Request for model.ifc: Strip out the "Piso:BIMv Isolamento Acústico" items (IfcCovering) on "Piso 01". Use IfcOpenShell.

First a look at what the model holds.

```python
import ifcopenshell
import ifcopenshell.util.element

model = ifcopenshell.open("model.ifc")
print(model.schema)
storey = next(s for s in model.by_type("IfcBuildingStorey") if s.Name == "Piso 01")
coverings = [e for e in ifcopenshell.util.element.get_decomposition(storey) if e.is_a("IfcCovering")]
seen = {}
for e in coverings:
    element_type = ifcopenshell.util.element.get_type(e)
    name = element_type.Name if element_type not in (None, e) else None
    seen[name] = seen.get(name, 0) + 1
for name, count in sorted(seen.items(), key=str):
    print(count, "x", name)
```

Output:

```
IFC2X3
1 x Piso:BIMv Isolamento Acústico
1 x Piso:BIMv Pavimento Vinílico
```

```python
import ifcopenshell
import ifcopenshell.api.root
import ifcopenshell.util.element

model = ifcopenshell.open("model.ifc")

storey = next(s for s in model.by_type("IfcBuildingStorey") if s.Name == "Piso 01")
coverings = [e for e in ifcopenshell.util.element.get_decomposition(storey) if e.is_a("IfcCovering")]
targets = [e for e in coverings if (t := ifcopenshell.util.element.get_type(e)) not in (None, e) and t.Name == "Piso:BIMv Isolamento Acústico"]

for e in targets:
    ifcopenshell.api.root.remove_product(model, product=e)
print(len(targets), "removed")

model.write("model_edited.ifc")
```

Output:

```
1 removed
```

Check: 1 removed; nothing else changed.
